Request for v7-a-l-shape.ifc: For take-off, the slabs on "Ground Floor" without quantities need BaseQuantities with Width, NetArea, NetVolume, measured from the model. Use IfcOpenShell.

First a look at what the model holds.

```python
import ifcopenshell
import ifcopenshell.util.element
import ifcopenshell.util.unit

model = ifcopenshell.open("v7-a-l-shape.ifc")
print(model.schema)
for unit_type in ("LENGTHUNIT", "AREAUNIT", "VOLUMEUNIT"):
    print(unit_type, ifcopenshell.util.unit.calculate_unit_scale(model, unit_type))
storey = next(s for s in model.by_type("IfcBuildingStorey") if s.Name == "Ground Floor")
slabs = [e for e in ifcopenshell.util.element.get_decomposition(storey) if e.is_a("IfcSlab")]
for e in sorted(slabs, key=lambda e: e.id()):
    print(e.id(), e.is_a(), e.Name, list(ifcopenshell.util.element.get_psets(e, qtos_only=True)), sep=" | ")
```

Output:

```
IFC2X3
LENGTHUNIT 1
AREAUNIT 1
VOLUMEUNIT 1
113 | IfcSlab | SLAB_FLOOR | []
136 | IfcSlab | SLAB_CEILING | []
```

```python
import ifcopenshell
import ifcopenshell.api.pset
import ifcopenshell.geom
import ifcopenshell.util.element
import ifcopenshell.util.shape
import ifcopenshell.util.unit

model = ifcopenshell.open("v7-a-l-shape.ifc")
unit_scale = ifcopenshell.util.unit.calculate_unit_scale(model)
area_scale = ifcopenshell.util.unit.calculate_unit_scale(model, "AREAUNIT")
volume_scale = ifcopenshell.util.unit.calculate_unit_scale(model, "VOLUMEUNIT")
settings = ifcopenshell.geom.settings()

storey = next(s for s in model.by_type("IfcBuildingStorey") if s.Name == "Ground Floor")
slabs = [e for e in ifcopenshell.util.element.get_decomposition(storey) if e.is_a("IfcSlab")]

for e in sorted(slabs, key=lambda e: e.id()):
    if ifcopenshell.util.element.get_psets(e, qtos_only=True, should_inherit=False):
        continue
    # Geometry comes back in metres, in the element's own axes.
    shape = ifcopenshell.geom.create_shape(settings, e)
    values = {
        "Width": ifcopenshell.util.shape.get_z(shape.geometry) / unit_scale,
        "NetArea": ifcopenshell.util.shape.get_footprint_area(shape.geometry) / area_scale,
        "NetVolume": ifcopenshell.util.shape.get_volume(shape.geometry) / volume_scale,
    }
    qto = ifcopenshell.api.pset.add_qto(model, product=e, name="BaseQuantities")
    ifcopenshell.api.pset.edit_qto(model, qto=qto, properties=values)
    print(e.id(), {k: round(v, 3) for k, v in values.items()})

model.write("v7-a-l-shape_rev.ifc")
```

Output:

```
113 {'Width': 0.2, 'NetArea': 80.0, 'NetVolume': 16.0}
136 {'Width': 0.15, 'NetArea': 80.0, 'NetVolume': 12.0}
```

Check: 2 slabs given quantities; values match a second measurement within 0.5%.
